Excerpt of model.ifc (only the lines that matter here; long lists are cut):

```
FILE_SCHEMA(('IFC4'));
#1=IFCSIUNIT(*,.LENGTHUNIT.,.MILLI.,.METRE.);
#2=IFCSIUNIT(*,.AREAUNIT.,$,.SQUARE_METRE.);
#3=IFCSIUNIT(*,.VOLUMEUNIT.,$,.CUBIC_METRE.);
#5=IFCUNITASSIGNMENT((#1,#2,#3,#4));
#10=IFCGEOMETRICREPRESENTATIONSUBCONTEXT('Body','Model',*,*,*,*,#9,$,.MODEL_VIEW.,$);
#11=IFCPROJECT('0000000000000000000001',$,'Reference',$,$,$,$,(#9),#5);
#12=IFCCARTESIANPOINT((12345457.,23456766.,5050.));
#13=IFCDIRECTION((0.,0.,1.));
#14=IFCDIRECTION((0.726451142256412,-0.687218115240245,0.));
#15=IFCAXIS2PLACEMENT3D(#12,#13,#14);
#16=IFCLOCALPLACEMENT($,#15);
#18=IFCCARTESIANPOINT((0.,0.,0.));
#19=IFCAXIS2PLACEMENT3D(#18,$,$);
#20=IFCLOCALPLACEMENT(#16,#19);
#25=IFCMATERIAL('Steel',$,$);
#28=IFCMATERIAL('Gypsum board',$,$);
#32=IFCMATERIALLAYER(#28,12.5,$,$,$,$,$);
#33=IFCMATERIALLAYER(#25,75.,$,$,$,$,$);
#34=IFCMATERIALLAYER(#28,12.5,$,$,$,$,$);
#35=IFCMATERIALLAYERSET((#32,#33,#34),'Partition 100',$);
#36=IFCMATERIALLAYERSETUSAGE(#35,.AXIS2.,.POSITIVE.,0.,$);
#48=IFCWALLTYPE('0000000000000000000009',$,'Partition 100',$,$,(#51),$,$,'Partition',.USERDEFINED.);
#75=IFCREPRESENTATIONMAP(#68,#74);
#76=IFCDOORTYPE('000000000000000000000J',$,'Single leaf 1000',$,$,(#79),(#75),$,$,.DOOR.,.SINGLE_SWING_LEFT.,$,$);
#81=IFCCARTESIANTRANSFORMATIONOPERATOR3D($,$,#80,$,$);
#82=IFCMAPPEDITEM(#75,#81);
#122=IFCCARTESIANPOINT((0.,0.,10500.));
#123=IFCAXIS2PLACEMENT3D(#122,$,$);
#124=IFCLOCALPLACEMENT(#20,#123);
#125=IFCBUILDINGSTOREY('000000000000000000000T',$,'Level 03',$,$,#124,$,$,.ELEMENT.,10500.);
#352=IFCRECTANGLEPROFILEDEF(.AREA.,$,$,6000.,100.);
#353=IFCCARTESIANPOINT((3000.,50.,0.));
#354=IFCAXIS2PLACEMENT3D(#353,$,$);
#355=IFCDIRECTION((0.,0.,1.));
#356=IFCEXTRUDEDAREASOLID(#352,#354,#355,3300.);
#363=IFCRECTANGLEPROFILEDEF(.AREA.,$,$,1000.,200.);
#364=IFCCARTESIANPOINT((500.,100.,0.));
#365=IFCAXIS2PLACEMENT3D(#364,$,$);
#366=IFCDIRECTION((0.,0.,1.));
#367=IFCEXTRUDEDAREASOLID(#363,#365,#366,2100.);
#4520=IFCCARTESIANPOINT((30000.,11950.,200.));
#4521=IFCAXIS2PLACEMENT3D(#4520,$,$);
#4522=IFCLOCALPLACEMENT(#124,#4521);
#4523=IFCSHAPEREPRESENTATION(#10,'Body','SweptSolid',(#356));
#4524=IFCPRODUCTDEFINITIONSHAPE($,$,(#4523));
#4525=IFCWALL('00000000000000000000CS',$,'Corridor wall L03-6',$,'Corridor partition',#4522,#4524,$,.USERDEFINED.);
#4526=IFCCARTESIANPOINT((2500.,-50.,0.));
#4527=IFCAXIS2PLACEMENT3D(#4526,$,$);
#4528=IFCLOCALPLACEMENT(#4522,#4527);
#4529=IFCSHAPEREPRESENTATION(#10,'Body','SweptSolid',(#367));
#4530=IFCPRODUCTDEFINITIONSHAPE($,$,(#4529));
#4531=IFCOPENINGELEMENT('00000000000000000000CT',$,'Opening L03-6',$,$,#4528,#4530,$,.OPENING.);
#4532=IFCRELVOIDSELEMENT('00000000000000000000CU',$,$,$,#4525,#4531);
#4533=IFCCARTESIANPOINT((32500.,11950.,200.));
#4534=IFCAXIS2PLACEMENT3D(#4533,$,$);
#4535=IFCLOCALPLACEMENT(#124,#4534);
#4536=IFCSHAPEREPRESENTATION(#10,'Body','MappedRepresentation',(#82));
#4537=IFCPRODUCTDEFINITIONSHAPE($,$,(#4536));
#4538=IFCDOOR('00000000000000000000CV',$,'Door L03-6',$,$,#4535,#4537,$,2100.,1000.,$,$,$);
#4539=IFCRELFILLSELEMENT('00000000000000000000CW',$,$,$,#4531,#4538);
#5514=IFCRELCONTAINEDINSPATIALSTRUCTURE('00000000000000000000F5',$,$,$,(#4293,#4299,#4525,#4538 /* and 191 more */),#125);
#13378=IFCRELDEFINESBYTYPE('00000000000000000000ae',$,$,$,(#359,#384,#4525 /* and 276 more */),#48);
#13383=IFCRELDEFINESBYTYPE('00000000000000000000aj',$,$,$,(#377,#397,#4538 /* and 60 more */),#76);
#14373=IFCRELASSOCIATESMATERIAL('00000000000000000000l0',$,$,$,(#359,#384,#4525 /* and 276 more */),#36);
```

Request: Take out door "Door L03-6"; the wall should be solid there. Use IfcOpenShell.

```python
import ifcopenshell
import ifcopenshell.api.feature
import ifcopenshell.api.root
import ifcopenshell.geom
import ifcopenshell.util.shape

model = ifcopenshell.open("model.ifc")
settings = ifcopenshell.geom.settings()


def volume(element):
    """Net volume in cubic metres, openings subtracted."""
    shape = ifcopenshell.geom.create_shape(settings, element)
    return ifcopenshell.util.shape.get_volume(shape.geometry)


door = model.by_id(4538)
opening = door.FillsVoids[0].RelatingOpeningElement
wall = opening.VoidsElements[0].RelatingBuildingElement
before = volume(wall)

ifcopenshell.api.root.remove_product(model, product=door)
ifcopenshell.api.feature.remove_feature(model, feature=opening)

after = volume(wall)

print(f"wall volume {before:.3f} -> {after:.3f} m3")

model.write("model_updated.ifc")
```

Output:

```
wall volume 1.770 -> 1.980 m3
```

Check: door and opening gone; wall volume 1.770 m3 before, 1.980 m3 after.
